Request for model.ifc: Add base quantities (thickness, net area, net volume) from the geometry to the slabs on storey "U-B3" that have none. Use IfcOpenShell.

First a look at what the model holds.

```python
import ifcopenshell
import ifcopenshell.util.element
import ifcopenshell.util.unit

model = ifcopenshell.open("model.ifc")
print(model.schema)
for unit_type in ("LENGTHUNIT", "AREAUNIT", "VOLUMEUNIT"):
    print(unit_type, ifcopenshell.util.unit.calculate_unit_scale(model, unit_type))
storey = next(s for s in model.by_type("IfcBuildingStorey") if s.Name == "U-B3")
slabs = [e for e in ifcopenshell.util.element.get_decomposition(storey) if e.is_a("IfcSlab")]
for e in sorted(slabs, key=lambda e: e.id()):
    print(e.id(), e.is_a(), e.Name, list(ifcopenshell.util.element.get_psets(e, qtos_only=True)), sep=" | ")
```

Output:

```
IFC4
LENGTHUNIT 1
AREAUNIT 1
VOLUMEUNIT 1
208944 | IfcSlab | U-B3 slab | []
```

```python
import ifcopenshell
import ifcopenshell.api.pset
import ifcopenshell.geom
import ifcopenshell.util.element
import ifcopenshell.util.shape
import ifcopenshell.util.unit

model = ifcopenshell.open("model.ifc")
unit_scale = ifcopenshell.util.unit.calculate_unit_scale(model)
area_scale = ifcopenshell.util.unit.calculate_unit_scale(model, "AREAUNIT")
volume_scale = ifcopenshell.util.unit.calculate_unit_scale(model, "VOLUMEUNIT")
settings = ifcopenshell.geom.settings()

storey = next(s for s in model.by_type("IfcBuildingStorey") if s.Name == "U-B3")
slabs = [e for e in ifcopenshell.util.element.get_decomposition(storey) if e.is_a("IfcSlab")]

for e in sorted(slabs, key=lambda e: e.id()):
    if ifcopenshell.util.element.get_psets(e, qtos_only=True, should_inherit=False):
        continue
    # Geometry comes back in metres, in the element's own axes.
    shape = ifcopenshell.geom.create_shape(settings, e)
    values = {
        "Width": ifcopenshell.util.shape.get_z(shape.geometry) / unit_scale,
        "NetArea": ifcopenshell.util.shape.get_footprint_area(shape.geometry) / area_scale,
        "NetVolume": ifcopenshell.util.shape.get_volume(shape.geometry) / volume_scale,
    }
    qto = ifcopenshell.api.pset.add_qto(model, product=e, name="Qto_SlabBaseQuantities")
    ifcopenshell.api.pset.edit_qto(model, qto=qto, properties=values)
    print(e.id(), {k: round(v, 3) for k, v in values.items()})

model.write("model_v2.ifc")
```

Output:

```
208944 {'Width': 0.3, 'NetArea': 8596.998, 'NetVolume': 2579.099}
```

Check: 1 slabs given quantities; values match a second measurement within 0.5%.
